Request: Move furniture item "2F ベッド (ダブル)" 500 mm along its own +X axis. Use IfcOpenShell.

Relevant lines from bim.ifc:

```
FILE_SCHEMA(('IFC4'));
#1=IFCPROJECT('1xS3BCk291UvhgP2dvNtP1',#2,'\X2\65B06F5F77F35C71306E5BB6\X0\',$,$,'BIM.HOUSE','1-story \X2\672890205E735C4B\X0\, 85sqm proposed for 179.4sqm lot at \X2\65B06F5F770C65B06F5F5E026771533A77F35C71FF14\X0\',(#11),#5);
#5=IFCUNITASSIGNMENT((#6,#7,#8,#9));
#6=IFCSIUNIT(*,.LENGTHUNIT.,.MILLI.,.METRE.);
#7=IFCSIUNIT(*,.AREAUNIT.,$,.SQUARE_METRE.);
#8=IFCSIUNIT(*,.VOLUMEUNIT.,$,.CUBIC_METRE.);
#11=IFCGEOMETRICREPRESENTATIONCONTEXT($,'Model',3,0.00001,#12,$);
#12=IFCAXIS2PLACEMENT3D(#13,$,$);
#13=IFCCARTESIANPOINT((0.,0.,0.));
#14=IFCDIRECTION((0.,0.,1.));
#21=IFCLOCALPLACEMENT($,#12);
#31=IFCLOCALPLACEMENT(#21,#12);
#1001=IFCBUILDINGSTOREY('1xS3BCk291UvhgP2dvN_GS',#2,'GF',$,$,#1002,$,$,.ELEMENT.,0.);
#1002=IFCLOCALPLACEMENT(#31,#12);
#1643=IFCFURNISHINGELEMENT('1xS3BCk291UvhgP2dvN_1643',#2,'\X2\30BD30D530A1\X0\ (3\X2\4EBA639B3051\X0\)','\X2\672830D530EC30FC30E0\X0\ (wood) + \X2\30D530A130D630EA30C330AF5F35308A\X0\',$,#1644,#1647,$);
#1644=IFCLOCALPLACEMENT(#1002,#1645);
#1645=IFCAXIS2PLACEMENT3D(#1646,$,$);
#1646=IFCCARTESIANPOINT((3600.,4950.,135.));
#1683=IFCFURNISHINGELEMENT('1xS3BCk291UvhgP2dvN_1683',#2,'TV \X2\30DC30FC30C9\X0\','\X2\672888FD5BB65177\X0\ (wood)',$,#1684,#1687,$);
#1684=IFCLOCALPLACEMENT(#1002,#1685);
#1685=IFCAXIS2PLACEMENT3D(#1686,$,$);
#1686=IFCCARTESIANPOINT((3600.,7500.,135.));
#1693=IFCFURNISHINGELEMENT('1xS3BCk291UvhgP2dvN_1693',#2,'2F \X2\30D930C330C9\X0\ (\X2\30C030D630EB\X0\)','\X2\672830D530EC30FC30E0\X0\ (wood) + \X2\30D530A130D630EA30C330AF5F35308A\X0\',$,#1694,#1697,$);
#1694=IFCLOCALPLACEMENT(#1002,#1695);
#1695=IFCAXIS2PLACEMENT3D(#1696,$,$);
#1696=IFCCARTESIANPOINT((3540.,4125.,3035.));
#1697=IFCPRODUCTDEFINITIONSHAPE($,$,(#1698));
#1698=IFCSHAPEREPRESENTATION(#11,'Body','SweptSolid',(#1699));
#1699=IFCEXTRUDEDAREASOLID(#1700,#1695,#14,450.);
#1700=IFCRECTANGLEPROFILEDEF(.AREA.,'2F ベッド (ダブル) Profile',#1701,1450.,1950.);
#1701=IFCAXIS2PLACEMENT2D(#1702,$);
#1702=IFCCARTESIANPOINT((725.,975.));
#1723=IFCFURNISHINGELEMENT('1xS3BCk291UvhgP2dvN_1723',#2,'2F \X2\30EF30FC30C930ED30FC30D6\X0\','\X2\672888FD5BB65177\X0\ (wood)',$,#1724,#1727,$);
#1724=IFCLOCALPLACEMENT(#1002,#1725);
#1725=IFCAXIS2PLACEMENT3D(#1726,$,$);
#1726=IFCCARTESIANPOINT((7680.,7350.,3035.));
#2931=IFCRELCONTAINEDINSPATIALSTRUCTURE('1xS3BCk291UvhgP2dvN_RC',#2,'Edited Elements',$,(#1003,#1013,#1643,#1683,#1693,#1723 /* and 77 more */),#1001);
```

```python
import ifcopenshell
import ifcopenshell.api.geometry
import ifcopenshell.util.placement

model = ifcopenshell.open("bim.ifc")

item = model.by_id(1693)
matrix = ifcopenshell.util.placement.get_local_placement(item.ObjectPlacement)
matrix[:3, 3] += matrix[:3, 0] * 500.0
ifcopenshell.api.geometry.edit_object_placement(model, product=item, matrix=matrix, is_si=False)

print(ifcopenshell.util.placement.get_local_placement(item.ObjectPlacement).round(3) + 0.0)

model.write("bim-out.ifc")
```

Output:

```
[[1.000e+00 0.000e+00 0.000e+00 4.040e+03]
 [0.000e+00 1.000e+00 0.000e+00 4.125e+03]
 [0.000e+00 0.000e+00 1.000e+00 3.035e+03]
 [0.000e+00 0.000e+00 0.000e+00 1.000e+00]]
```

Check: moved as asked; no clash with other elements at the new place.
